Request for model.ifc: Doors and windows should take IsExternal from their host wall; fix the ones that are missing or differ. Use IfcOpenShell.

First a look at what the model holds.

```python
import ifcopenshell
import ifcopenshell.util.element

model = ifcopenshell.open("model.ifc")
print(model.schema)
seen = {}
for e in model.by_type("IfcDoor") + model.by_type("IfcWindow"):
    if not e.FillsVoids:
        continue
    host = e.FillsVoids[0].RelatingOpeningElement.VoidsElements[0].RelatingBuildingElement
    own = ifcopenshell.util.element.get_pset(e, f"Pset_{e.is_a()[3:].removesuffix('StandardCase')}Common", "IsExternal")
    wall = ifcopenshell.util.element.get_pset(host, "Pset_WallCommon", "IsExternal")
    seen[e.is_a(), own, wall] = seen.get((e.is_a(), own, wall), 0) + 1
for (cls, own, wall), count in sorted(seen.items(), key=str):
    print(count, cls, "IsExternal:", own, "| host wall:", wall)
```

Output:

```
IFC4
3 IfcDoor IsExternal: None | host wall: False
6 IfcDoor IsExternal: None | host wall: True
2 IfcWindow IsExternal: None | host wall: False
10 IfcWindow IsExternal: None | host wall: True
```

```python
import ifcopenshell
import ifcopenshell.api.pset
import ifcopenshell.util.element

model = ifcopenshell.open("model.ifc")

count = 0
for ifc_class, pset_name in (("IfcDoor", "Pset_DoorCommon"), ("IfcWindow", "Pset_WindowCommon")):
    for e in model.by_type(ifc_class):
        if not e.FillsVoids:
            continue
        host = e.FillsVoids[0].RelatingOpeningElement.VoidsElements[0].RelatingBuildingElement
        external = ifcopenshell.util.element.get_pset(host, "Pset_WallCommon", "IsExternal")
        if external is None or ifcopenshell.util.element.get_pset(e, pset_name, "IsExternal") == external:
            continue
        pset = ifcopenshell.api.pset.add_pset(model, product=e, name=pset_name)
        ifcopenshell.api.pset.edit_pset(model, pset=pset, properties={"IsExternal": external})
        count += 1

print(count, "updated")

model.write("model_v2.ifc")
```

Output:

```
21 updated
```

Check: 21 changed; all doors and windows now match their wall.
